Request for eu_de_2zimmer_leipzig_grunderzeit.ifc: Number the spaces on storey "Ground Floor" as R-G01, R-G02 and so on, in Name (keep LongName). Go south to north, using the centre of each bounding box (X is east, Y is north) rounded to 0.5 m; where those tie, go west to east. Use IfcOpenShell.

First a look at what the model holds.

```python
import ifcopenshell
import ifcopenshell.util.element
import ifcopenshell.util.placement

model = ifcopenshell.open("eu_de_2zimmer_leipzig_grunderzeit.ifc")
print(model.schema)
storey = next(s for s in model.by_type("IfcBuildingStorey") if s.Name == "Ground Floor")
spaces = [e for e in ifcopenshell.util.element.get_decomposition(storey) if e.is_a("IfcSpace")]
for e in sorted(spaces, key=lambda e: e.id()):
    origin = ifcopenshell.util.placement.get_local_placement(e.ObjectPlacement)[:3, 3]
    print(e.id(), e.Name, e.LongName, origin.round(2) + 0.0, sep=" | ")
```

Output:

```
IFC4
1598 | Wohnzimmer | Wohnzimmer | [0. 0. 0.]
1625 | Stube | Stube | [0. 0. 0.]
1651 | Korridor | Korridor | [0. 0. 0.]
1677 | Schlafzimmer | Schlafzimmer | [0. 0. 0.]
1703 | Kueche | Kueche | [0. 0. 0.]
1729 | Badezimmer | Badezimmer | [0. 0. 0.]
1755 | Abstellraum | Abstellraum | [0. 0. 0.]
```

```python
import ifcopenshell
import ifcopenshell.geom
import ifcopenshell.util.element
import ifcopenshell.util.shape

model = ifcopenshell.open("eu_de_2zimmer_leipzig_grunderzeit.ifc")
settings = ifcopenshell.geom.settings()
settings.set("use-world-coords", True)


def centre(element):
    shape = ifcopenshell.geom.create_shape(settings, element)
    return ifcopenshell.util.shape.get_bbox_centroid(shape.geometry)


storey = next(s for s in model.by_type("IfcBuildingStorey") if s.Name == "Ground Floor")
spaces = [e for e in ifcopenshell.util.element.get_decomposition(storey) if e.is_a("IfcSpace")]

# Insertion points can sit at a corner or the storey origin, so sort by the geometry (in metres).
centres = {e: centre(e) for e in spaces}
spaces.sort(key=lambda e: (round(centres[e][1] / 0.5), centres[e][0]))

for i, e in enumerate(spaces, start=1):
    number = f"R-G{i:02d}"
    e.Name = number
    print(e.id(), number)

model.write("eu_de_2zimmer_leipzig_grunderzeit_v2.ifc")
```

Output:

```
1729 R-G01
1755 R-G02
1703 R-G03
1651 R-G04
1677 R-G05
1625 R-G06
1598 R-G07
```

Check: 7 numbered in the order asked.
